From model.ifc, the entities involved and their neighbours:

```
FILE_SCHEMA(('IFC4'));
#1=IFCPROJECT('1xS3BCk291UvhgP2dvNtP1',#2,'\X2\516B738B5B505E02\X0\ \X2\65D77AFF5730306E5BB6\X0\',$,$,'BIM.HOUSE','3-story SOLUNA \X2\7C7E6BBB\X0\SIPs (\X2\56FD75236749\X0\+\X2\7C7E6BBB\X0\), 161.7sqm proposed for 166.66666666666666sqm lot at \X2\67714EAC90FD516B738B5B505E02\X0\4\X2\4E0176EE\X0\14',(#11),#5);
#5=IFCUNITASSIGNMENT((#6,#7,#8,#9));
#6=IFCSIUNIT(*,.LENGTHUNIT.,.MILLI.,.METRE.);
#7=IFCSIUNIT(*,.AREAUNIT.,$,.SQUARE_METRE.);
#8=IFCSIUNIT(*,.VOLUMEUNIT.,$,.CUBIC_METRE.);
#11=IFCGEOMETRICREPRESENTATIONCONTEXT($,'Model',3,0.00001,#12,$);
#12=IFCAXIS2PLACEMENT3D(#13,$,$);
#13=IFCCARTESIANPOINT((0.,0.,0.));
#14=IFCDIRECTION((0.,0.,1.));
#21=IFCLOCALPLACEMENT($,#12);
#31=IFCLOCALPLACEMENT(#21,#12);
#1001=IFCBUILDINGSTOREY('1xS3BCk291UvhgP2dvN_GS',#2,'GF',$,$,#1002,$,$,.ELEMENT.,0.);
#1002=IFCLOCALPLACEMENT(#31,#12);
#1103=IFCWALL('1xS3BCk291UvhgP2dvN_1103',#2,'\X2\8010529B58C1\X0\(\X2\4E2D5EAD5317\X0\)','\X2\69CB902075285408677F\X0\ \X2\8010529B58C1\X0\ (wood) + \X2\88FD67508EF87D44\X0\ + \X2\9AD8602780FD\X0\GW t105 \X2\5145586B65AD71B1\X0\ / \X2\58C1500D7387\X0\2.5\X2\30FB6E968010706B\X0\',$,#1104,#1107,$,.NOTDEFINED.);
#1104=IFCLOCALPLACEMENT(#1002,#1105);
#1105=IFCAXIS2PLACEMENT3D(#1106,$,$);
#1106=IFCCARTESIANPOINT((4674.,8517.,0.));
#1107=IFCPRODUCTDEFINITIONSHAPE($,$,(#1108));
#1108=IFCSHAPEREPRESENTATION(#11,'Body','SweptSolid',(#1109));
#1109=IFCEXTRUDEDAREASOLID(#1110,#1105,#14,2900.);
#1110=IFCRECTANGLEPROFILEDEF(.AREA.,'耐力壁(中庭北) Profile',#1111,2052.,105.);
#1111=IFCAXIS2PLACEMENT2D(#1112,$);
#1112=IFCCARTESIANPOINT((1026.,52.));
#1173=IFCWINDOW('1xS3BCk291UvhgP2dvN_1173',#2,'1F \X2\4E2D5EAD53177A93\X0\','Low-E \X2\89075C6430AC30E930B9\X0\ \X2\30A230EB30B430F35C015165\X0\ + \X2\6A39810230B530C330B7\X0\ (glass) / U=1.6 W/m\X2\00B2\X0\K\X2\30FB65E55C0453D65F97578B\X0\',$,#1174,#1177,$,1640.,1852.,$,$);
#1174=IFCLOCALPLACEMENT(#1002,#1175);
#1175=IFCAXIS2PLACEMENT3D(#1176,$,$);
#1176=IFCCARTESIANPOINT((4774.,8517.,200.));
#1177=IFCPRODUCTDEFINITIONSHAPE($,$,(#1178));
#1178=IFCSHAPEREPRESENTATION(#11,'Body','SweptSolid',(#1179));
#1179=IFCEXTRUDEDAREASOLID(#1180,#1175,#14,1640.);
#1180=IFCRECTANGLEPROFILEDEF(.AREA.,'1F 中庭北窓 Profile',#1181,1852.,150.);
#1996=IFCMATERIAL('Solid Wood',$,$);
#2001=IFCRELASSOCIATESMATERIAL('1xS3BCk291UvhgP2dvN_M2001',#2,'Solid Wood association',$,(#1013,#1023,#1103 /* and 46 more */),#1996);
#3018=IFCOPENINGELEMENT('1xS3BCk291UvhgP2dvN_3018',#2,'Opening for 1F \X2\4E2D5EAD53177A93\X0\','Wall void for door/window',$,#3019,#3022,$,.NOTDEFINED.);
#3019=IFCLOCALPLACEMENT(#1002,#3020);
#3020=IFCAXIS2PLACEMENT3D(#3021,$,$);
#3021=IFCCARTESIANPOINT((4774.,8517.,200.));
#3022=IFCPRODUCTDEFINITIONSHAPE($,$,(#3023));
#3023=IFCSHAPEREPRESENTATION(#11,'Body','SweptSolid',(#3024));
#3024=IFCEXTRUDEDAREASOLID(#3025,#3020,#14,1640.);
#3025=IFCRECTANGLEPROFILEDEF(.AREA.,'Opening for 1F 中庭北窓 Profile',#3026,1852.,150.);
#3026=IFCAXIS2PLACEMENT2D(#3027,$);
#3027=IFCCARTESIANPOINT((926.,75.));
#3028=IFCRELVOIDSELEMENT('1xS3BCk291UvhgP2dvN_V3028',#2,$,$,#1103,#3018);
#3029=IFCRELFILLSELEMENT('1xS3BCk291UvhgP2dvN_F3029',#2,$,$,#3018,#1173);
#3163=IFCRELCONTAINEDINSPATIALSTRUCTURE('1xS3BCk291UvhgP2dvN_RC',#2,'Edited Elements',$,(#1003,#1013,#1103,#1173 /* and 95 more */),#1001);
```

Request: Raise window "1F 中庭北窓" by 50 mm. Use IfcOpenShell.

```python
import numpy as np
import ifcopenshell
import ifcopenshell.api.geometry
import ifcopenshell.util.placement
import ifcopenshell.util.unit

model = ifcopenshell.open("model.ifc")
unit_scale = ifcopenshell.util.unit.calculate_unit_scale(model)

window = model.by_id(1173)
opening = window.FillsVoids[0].RelatingOpeningElement
dz = 0.05 / unit_scale

shift = np.array([0.0, 0.0, dz])
# The window is not placed relative to its opening, so move both.
for product in (opening, window):
    matrix = ifcopenshell.util.placement.get_local_placement(product.ObjectPlacement)
    matrix[:3, 3] += shift
    ifcopenshell.api.geometry.edit_object_placement(model, product=product, matrix=matrix, is_si=False)

print(f"moved by {dz * unit_scale:+.3f} m")

model.write("model-out.ifc")
```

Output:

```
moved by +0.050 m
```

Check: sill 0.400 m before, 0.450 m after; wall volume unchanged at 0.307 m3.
